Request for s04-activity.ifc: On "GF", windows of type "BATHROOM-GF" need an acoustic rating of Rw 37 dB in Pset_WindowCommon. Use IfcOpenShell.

First a look at what the model holds.

```python
import ifcopenshell
import ifcopenshell.util.element

model = ifcopenshell.open("s04-activity.ifc")
print(model.schema)
storey = next(s for s in model.by_type("IfcBuildingStorey") if s.Name == "GF")
windows = [e for e in ifcopenshell.util.element.get_decomposition(storey) if e.is_a("IfcWindow")]
seen = {}
for e in windows:
    element_type = ifcopenshell.util.element.get_type(e)
    key = (element_type.Name if element_type != e and element_type else None, ifcopenshell.util.element.get_pset(e, "Pset_WindowCommon", "AcousticRating"))
    seen[key] = seen.get(key, 0) + 1
for (name, value), count in sorted(seen.items(), key=str):
    print(count, "x", name, "|", value)
```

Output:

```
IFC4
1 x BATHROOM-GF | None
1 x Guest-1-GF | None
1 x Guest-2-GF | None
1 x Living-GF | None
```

```python
import ifcopenshell
import ifcopenshell.api.pset
import ifcopenshell.util.element

model = ifcopenshell.open("s04-activity.ifc")

storey = next(s for s in model.by_type("IfcBuildingStorey") if s.Name == "GF")
windows = [e for e in ifcopenshell.util.element.get_decomposition(storey) if e.is_a("IfcWindow")]

count = 0
for e in windows:
    element_type = ifcopenshell.util.element.get_type(e)
    if element_type in (None, e) or element_type.Name != "BATHROOM-GF":
        continue
    # add_pset returns the element's existing set when there is one.
    pset = ifcopenshell.api.pset.add_pset(model, product=e, name="Pset_WindowCommon")
    ifcopenshell.api.pset.edit_pset(model, pset=pset, properties={"AcousticRating": "Rw 37 dB"})
    count += 1

print(count, "windows updated")

model.write("s04-activity_edited.ifc")
```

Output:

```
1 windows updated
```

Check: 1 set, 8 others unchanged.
